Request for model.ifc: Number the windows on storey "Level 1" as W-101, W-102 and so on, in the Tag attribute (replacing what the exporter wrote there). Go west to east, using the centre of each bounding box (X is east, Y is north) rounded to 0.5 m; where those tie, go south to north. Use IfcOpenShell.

First a look at what the model holds.

```python
import ifcopenshell
import ifcopenshell.util.element
import ifcopenshell.util.placement

model = ifcopenshell.open("model.ifc")
print(model.schema)
storey = next(s for s in model.by_type("IfcBuildingStorey") if s.Name == "Level 1")
windows = [e for e in ifcopenshell.util.element.get_decomposition(storey) if e.is_a("IfcWindow")]
for e in sorted(windows, key=lambda e: e.id()):
    origin = ifcopenshell.util.placement.get_local_placement(e.ObjectPlacement)[:3, 3]
    print(e.id(), e.Tag, e.Name, origin.round(2) + 0.0, sep=" | ")
```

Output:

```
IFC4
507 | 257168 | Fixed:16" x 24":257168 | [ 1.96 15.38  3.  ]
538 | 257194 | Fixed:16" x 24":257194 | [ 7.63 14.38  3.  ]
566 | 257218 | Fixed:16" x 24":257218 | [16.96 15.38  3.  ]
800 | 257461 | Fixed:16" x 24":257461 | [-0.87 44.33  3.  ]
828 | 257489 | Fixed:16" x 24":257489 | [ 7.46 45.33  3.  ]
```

```python
import ifcopenshell
import ifcopenshell.geom
import ifcopenshell.util.element
import ifcopenshell.util.shape

model = ifcopenshell.open("model.ifc")
settings = ifcopenshell.geom.settings()
settings.set("use-world-coords", True)


def centre(element):
    shape = ifcopenshell.geom.create_shape(settings, element)
    return ifcopenshell.util.shape.get_bbox_centroid(shape.geometry)


storey = next(s for s in model.by_type("IfcBuildingStorey") if s.Name == "Level 1")
windows = [e for e in ifcopenshell.util.element.get_decomposition(storey) if e.is_a("IfcWindow")]

# Insertion points can sit at a corner or the storey origin, so sort by the geometry (in metres).
centres = {e: centre(e) for e in windows}
windows.sort(key=lambda e: (round(centres[e][0] / 0.5), centres[e][1]))

for i, e in enumerate(windows, start=1):
    number = f"W-1{i:02d}"
    e.Tag = number
    print(e.id(), number)

model.write("model-out.ifc")
```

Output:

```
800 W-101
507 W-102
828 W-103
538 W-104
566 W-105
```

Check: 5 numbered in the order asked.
